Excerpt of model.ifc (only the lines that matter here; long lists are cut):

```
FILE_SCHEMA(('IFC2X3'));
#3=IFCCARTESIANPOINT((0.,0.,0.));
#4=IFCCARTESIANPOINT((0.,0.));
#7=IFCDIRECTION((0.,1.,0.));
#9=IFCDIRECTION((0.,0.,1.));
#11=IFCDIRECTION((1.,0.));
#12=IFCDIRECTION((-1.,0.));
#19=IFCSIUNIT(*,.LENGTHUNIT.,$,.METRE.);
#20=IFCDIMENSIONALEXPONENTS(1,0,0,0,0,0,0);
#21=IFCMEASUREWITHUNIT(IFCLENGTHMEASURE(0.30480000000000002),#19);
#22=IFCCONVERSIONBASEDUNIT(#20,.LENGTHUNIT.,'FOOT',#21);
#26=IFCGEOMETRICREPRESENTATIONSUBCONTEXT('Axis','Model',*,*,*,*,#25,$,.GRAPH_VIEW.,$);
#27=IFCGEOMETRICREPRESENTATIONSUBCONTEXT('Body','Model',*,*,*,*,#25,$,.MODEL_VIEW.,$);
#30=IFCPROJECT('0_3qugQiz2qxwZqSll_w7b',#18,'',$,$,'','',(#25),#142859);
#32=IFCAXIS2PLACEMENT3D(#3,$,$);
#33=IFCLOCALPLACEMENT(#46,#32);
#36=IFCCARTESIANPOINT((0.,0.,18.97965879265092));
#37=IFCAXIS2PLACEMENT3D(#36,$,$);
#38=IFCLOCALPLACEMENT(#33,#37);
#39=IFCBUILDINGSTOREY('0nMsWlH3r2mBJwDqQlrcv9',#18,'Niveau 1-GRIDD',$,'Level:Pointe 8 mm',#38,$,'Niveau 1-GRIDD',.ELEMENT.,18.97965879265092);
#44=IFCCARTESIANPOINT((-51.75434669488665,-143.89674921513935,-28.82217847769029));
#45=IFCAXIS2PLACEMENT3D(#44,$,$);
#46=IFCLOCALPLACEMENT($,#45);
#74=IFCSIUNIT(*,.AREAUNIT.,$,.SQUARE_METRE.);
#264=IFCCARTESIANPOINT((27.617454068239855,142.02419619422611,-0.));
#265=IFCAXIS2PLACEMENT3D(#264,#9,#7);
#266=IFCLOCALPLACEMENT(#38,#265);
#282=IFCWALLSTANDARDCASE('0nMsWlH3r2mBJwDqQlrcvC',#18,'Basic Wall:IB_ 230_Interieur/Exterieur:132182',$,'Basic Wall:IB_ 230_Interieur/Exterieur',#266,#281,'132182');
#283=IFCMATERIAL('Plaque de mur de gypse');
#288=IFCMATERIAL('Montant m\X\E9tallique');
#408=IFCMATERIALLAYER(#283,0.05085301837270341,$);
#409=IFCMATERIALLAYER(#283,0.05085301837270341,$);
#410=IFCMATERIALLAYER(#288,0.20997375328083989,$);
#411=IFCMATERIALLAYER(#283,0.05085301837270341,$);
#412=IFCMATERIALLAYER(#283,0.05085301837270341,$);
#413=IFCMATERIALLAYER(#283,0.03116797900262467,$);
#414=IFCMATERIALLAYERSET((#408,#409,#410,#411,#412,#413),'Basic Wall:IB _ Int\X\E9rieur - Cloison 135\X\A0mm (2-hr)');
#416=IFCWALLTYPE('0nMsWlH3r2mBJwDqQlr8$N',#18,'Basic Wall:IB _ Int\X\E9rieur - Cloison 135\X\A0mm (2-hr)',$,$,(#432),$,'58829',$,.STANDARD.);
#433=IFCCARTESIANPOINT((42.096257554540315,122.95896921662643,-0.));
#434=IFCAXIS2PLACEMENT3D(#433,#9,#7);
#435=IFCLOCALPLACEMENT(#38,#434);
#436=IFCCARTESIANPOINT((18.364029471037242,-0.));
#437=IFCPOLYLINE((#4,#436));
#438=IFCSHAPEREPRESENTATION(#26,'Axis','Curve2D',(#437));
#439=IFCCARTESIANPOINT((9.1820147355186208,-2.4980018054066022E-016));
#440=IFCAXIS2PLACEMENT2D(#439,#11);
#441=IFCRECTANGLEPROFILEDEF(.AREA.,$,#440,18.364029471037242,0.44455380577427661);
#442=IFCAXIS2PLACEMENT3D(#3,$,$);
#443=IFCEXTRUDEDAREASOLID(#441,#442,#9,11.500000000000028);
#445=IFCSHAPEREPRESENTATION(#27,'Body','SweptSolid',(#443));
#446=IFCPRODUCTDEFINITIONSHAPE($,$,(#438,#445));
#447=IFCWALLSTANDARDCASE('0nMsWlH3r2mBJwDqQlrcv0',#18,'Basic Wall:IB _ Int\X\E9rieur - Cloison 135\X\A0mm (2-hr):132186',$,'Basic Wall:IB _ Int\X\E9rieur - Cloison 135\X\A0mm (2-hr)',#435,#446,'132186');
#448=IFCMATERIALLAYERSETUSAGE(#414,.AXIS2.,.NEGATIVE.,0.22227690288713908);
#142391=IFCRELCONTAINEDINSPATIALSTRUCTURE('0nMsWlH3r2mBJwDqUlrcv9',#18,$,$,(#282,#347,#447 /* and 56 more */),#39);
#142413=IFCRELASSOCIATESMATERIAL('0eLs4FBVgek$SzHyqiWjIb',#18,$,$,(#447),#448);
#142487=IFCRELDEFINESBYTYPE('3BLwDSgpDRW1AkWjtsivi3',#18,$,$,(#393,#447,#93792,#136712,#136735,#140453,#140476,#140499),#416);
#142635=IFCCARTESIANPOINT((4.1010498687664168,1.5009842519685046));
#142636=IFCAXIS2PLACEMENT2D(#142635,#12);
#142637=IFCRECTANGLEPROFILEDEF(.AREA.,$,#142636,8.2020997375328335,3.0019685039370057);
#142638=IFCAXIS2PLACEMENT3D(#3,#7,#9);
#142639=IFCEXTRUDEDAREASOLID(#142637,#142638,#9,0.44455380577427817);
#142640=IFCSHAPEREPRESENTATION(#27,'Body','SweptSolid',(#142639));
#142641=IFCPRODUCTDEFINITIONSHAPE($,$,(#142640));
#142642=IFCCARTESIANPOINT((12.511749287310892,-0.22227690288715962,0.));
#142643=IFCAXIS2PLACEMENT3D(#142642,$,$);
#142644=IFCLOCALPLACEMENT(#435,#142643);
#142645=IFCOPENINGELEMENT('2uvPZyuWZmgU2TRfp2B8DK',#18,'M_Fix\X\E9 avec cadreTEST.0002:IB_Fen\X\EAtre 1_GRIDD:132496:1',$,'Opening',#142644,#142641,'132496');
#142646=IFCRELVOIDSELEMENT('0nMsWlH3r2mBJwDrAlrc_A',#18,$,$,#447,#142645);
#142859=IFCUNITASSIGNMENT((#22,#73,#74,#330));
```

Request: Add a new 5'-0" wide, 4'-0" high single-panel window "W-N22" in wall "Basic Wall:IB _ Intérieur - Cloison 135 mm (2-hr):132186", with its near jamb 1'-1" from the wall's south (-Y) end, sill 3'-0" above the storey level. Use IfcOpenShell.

```python
import numpy as np
import ifcopenshell
import ifcopenshell.api.feature
import ifcopenshell.api.geometry
import ifcopenshell.api.root
import ifcopenshell.api.spatial
import ifcopenshell.api.type
import ifcopenshell.geom
import ifcopenshell.util.element
import ifcopenshell.util.placement
import ifcopenshell.util.representation
import ifcopenshell.util.shape
import ifcopenshell.util.unit

model = ifcopenshell.open("model.ifc")
unit_scale = ifcopenshell.util.unit.calculate_unit_scale(model)
settings = ifcopenshell.geom.settings()


def volume(element):
    """Net volume in cubic metres, openings subtracted."""
    shape = ifcopenshell.geom.create_shape(settings, element)
    return ifcopenshell.util.shape.get_volume(shape.geometry)


wall = model.by_guid("0nMsWlH3r2mBJwDqQlrcv0")
storey = ifcopenshell.util.element.get_container(wall, ifc_class="IfcBuildingStorey")
context = ifcopenshell.util.representation.get_context(model, "Model", "Body", "MODEL_VIEW")
before = volume(wall)

width, height, from_end, sill = 1.524, 1.2192, 0.3302, 0.9144  # metres

# The wall runs along its own X axis, and the end named is its -X end.
wall_shape = ifcopenshell.geom.create_shape(settings, wall)
x, y, z = ifcopenshell.util.shape.get_vertices(wall_shape.geometry).T
start = x.min() + from_end
face, thickness = float(y.min()), float(y.max() - y.min())
wall_matrix = ifcopenshell.util.placement.get_local_placement(wall.ObjectPlacement)
level = ifcopenshell.util.placement.get_local_placement(storey.ObjectPlacement)[2, 3]


def in_wall(x, y):
    """Placement at x, y metres in the wall's axes, at sill height."""
    matrix = wall_matrix.copy()
    matrix[:, 3] = wall_matrix @ np.array([x / unit_scale, y / unit_scale, 0.0, 1.0])
    matrix[2, 3] = level + sill / unit_scale
    return matrix


# Opening: a box that overshoots both wall faces by 50 mm.
opening = ifcopenshell.api.root.create_entity(model, ifc_class="IfcOpeningElement")
box = ifcopenshell.api.geometry.add_wall_representation(
    model, context=context, length=width, height=height, thickness=thickness + 0.1
)
ifcopenshell.api.geometry.assign_representation(model, product=opening, representation=box)
ifcopenshell.api.geometry.edit_object_placement(model, product=opening, matrix=in_wall(start, face - 0.05), is_si=False)
ifcopenshell.api.feature.add_feature(model, feature=opening, element=wall)

window = ifcopenshell.api.root.create_entity(model, ifc_class="IfcWindow", name="W-N22")
window.OverallWidth, window.OverallHeight = width / unit_scale, height / unit_scale
body = ifcopenshell.api.geometry.add_window_representation(
    model,
    context=context,
    overall_width=window.OverallWidth,
    overall_height=window.OverallHeight,
    partition_type="SINGLE_PANEL",
)
ifcopenshell.api.geometry.assign_representation(model, product=window, representation=body)
ifcopenshell.api.spatial.assign_container(model, products=[window], relating_structure=storey)
fills = ifcopenshell.api.feature.add_filling(model, opening=opening, element=window)
fills.OwnerHistory = window.OwnerHistory  # required in IFC2X3

# IFC2X3 keeps the operation on the window style.
style = ifcopenshell.api.root.create_entity(model, ifc_class="IfcWindowStyle", name="W-N22")
style.OperationType, style.ConstructionType = "SINGLE_PANEL", "NOTDEFINED"
style.ParameterTakesPrecedence = style.Sizeable = False
ifcopenshell.api.type.assign_type(model, related_objects=[window], relating_type=style)

# Centre the window in the wall's thickness.
ifcopenshell.api.geometry.edit_object_placement(model, product=window, matrix=in_wall(start, face), is_si=False)
window_shape = ifcopenshell.geom.create_shape(settings, window)
depth = ifcopenshell.util.shape.get_vertices(window_shape.geometry)[:, 1]
offset = face + thickness / 2 - (depth.min() + depth.max()) / 2
ifcopenshell.api.geometry.edit_object_placement(model, product=window, matrix=in_wall(start, offset), is_si=False)

after = volume(wall)

print(f"wall volume {before:.3f} -> {after:.3f} m3")

model.write("model_edited.ifc")
```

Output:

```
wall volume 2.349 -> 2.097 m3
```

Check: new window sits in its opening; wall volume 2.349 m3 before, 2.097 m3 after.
